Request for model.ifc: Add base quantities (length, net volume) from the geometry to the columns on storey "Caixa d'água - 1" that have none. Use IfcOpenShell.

First a look at what the model holds.

```python
import ifcopenshell
import ifcopenshell.util.element
import ifcopenshell.util.unit

model = ifcopenshell.open("model.ifc")
print(model.schema)
for unit_type in ("LENGTHUNIT", "AREAUNIT", "VOLUMEUNIT"):
    print(unit_type, ifcopenshell.util.unit.calculate_unit_scale(model, unit_type))
storey = next(s for s in model.by_type("IfcBuildingStorey") if s.Name == "Caixa d'água - 1")
columns = [e for e in ifcopenshell.util.element.get_decomposition(storey) if e.is_a("IfcColumn")]
for e in sorted(columns, key=lambda e: e.id()):
    print(e.id(), e.is_a(), e.Name, list(ifcopenshell.util.element.get_psets(e, qtos_only=True)), sep=" | ")
```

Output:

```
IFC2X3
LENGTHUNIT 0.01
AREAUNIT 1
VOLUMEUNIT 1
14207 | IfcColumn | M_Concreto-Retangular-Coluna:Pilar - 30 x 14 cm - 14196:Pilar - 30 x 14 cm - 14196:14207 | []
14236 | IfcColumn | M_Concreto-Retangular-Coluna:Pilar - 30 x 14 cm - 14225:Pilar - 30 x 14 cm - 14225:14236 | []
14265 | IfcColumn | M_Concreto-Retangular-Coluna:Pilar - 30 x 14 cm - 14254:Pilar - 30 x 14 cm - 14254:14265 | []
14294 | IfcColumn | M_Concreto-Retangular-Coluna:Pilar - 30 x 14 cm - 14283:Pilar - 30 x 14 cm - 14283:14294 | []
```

```python
import ifcopenshell
import ifcopenshell.api.pset
import ifcopenshell.geom
import ifcopenshell.util.element
import ifcopenshell.util.shape
import ifcopenshell.util.unit

model = ifcopenshell.open("model.ifc")
unit_scale = ifcopenshell.util.unit.calculate_unit_scale(model)
volume_scale = ifcopenshell.util.unit.calculate_unit_scale(model, "VOLUMEUNIT")
settings = ifcopenshell.geom.settings()

storey = next(s for s in model.by_type("IfcBuildingStorey") if s.Name == "Caixa d'água - 1")
columns = [e for e in ifcopenshell.util.element.get_decomposition(storey) if e.is_a("IfcColumn")]

for e in sorted(columns, key=lambda e: e.id()):
    if ifcopenshell.util.element.get_psets(e, qtos_only=True, should_inherit=False):
        continue
    # Geometry comes back in metres, in the element's own axes.
    shape = ifcopenshell.geom.create_shape(settings, e)
    values = {
        "Length": ifcopenshell.util.shape.get_z(shape.geometry) / unit_scale,
        "NetVolume": ifcopenshell.util.shape.get_volume(shape.geometry) / volume_scale,
    }
    qto = ifcopenshell.api.pset.add_qto(model, product=e, name="BaseQuantities")
    ifcopenshell.api.pset.edit_qto(model, qto=qto, properties=values)
    print(e.id(), {k: round(v, 3) for k, v in values.items()})

model.write("model-out.ifc")
```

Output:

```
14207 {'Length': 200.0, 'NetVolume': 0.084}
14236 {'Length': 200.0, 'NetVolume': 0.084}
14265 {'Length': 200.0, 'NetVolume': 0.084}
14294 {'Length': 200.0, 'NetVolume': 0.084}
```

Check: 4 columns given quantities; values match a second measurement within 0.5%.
